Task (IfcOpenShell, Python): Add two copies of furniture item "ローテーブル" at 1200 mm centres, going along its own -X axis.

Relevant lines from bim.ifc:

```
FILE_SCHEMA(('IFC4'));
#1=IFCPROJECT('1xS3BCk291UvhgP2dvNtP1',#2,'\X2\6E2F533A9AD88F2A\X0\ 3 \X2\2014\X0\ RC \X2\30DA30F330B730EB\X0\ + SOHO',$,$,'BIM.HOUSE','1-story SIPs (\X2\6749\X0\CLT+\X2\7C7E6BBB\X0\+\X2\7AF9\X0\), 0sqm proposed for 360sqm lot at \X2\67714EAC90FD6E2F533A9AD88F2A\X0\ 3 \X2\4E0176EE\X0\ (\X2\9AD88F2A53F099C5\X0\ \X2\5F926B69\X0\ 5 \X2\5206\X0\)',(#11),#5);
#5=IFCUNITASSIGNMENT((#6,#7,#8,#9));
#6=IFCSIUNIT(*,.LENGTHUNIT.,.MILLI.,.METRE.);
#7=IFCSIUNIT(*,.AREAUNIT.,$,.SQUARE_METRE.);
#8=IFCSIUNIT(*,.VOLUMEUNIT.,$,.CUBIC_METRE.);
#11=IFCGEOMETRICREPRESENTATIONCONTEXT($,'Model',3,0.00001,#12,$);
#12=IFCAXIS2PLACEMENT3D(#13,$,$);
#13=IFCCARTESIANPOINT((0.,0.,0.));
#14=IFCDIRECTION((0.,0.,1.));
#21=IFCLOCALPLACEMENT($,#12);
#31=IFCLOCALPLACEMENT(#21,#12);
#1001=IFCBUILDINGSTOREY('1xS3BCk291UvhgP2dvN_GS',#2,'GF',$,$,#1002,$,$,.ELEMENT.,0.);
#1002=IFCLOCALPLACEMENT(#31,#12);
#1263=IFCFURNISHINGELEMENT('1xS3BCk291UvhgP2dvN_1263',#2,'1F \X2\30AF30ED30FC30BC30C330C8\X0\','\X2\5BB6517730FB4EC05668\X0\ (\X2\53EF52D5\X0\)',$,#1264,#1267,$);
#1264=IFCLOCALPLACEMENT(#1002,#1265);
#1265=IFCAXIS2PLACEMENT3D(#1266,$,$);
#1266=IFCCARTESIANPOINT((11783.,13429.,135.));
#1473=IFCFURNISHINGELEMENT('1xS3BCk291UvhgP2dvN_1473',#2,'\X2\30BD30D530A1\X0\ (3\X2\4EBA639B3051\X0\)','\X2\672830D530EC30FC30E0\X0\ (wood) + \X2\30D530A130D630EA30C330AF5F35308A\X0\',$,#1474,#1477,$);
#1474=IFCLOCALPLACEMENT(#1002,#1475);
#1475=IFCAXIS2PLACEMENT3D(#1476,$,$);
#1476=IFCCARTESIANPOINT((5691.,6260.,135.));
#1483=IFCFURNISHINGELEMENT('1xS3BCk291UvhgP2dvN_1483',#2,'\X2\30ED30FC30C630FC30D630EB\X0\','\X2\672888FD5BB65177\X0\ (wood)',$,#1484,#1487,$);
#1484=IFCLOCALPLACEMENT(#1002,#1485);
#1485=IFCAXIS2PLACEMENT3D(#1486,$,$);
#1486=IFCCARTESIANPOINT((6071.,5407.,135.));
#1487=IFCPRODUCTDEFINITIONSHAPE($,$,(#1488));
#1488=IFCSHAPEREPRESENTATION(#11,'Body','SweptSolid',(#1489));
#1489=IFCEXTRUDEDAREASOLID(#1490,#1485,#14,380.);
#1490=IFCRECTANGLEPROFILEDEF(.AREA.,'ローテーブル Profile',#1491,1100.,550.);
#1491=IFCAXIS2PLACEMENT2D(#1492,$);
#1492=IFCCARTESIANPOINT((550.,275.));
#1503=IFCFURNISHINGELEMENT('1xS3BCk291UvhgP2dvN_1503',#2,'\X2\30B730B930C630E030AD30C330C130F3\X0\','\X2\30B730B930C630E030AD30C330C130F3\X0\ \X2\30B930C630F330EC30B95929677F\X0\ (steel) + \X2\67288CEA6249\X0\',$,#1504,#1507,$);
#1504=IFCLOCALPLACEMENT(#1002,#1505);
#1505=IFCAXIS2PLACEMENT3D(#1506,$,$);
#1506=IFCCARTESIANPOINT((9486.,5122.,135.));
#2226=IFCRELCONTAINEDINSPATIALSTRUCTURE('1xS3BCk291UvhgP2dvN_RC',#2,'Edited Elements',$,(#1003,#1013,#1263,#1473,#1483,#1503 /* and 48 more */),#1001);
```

```python
import ifcopenshell
import ifcopenshell.api.geometry
import ifcopenshell.api.root
import ifcopenshell.util.element
import ifcopenshell.util.placement

model = ifcopenshell.open("bim.ifc")


def reuse_history(source, copy):
    """copy_class also copies each property set's owner history, people and application; keep the originals."""
    for rel in copy.IsDefinedBy:
        if rel.is_a("IfcRelDefinesByProperties") and (history := rel.RelatingPropertyDefinition.OwnerHistory):
            rel.RelatingPropertyDefinition.OwnerHistory = source.OwnerHistory
            ifcopenshell.util.element.remove_deep2(model, history)


source = model.by_guid("1xS3BCk291UvhgP2dvN_1483")
base = ifcopenshell.util.placement.get_local_placement(source.ObjectPlacement)
step = -base[:3, 0] * 1200.0

for i in range(1, 3):
    copy = ifcopenshell.api.root.copy_class(model, product=source)
    copy.Representation = ifcopenshell.util.element.copy_deep(
        model, source.Representation, exclude=["IfcGeometricRepresentationContext", "IfcRepresentationMap"]
    )
    reuse_history(source, copy)
    matrix = base.copy()
    matrix[:3, 3] += i * step
    print("added at", matrix[:3, 3].round(3) + 0.0)
    ifcopenshell.api.geometry.edit_object_placement(model, product=copy, matrix=matrix, is_si=False)

model.write("bim_v2.ifc")
```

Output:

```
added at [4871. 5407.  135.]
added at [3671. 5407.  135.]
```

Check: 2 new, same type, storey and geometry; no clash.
